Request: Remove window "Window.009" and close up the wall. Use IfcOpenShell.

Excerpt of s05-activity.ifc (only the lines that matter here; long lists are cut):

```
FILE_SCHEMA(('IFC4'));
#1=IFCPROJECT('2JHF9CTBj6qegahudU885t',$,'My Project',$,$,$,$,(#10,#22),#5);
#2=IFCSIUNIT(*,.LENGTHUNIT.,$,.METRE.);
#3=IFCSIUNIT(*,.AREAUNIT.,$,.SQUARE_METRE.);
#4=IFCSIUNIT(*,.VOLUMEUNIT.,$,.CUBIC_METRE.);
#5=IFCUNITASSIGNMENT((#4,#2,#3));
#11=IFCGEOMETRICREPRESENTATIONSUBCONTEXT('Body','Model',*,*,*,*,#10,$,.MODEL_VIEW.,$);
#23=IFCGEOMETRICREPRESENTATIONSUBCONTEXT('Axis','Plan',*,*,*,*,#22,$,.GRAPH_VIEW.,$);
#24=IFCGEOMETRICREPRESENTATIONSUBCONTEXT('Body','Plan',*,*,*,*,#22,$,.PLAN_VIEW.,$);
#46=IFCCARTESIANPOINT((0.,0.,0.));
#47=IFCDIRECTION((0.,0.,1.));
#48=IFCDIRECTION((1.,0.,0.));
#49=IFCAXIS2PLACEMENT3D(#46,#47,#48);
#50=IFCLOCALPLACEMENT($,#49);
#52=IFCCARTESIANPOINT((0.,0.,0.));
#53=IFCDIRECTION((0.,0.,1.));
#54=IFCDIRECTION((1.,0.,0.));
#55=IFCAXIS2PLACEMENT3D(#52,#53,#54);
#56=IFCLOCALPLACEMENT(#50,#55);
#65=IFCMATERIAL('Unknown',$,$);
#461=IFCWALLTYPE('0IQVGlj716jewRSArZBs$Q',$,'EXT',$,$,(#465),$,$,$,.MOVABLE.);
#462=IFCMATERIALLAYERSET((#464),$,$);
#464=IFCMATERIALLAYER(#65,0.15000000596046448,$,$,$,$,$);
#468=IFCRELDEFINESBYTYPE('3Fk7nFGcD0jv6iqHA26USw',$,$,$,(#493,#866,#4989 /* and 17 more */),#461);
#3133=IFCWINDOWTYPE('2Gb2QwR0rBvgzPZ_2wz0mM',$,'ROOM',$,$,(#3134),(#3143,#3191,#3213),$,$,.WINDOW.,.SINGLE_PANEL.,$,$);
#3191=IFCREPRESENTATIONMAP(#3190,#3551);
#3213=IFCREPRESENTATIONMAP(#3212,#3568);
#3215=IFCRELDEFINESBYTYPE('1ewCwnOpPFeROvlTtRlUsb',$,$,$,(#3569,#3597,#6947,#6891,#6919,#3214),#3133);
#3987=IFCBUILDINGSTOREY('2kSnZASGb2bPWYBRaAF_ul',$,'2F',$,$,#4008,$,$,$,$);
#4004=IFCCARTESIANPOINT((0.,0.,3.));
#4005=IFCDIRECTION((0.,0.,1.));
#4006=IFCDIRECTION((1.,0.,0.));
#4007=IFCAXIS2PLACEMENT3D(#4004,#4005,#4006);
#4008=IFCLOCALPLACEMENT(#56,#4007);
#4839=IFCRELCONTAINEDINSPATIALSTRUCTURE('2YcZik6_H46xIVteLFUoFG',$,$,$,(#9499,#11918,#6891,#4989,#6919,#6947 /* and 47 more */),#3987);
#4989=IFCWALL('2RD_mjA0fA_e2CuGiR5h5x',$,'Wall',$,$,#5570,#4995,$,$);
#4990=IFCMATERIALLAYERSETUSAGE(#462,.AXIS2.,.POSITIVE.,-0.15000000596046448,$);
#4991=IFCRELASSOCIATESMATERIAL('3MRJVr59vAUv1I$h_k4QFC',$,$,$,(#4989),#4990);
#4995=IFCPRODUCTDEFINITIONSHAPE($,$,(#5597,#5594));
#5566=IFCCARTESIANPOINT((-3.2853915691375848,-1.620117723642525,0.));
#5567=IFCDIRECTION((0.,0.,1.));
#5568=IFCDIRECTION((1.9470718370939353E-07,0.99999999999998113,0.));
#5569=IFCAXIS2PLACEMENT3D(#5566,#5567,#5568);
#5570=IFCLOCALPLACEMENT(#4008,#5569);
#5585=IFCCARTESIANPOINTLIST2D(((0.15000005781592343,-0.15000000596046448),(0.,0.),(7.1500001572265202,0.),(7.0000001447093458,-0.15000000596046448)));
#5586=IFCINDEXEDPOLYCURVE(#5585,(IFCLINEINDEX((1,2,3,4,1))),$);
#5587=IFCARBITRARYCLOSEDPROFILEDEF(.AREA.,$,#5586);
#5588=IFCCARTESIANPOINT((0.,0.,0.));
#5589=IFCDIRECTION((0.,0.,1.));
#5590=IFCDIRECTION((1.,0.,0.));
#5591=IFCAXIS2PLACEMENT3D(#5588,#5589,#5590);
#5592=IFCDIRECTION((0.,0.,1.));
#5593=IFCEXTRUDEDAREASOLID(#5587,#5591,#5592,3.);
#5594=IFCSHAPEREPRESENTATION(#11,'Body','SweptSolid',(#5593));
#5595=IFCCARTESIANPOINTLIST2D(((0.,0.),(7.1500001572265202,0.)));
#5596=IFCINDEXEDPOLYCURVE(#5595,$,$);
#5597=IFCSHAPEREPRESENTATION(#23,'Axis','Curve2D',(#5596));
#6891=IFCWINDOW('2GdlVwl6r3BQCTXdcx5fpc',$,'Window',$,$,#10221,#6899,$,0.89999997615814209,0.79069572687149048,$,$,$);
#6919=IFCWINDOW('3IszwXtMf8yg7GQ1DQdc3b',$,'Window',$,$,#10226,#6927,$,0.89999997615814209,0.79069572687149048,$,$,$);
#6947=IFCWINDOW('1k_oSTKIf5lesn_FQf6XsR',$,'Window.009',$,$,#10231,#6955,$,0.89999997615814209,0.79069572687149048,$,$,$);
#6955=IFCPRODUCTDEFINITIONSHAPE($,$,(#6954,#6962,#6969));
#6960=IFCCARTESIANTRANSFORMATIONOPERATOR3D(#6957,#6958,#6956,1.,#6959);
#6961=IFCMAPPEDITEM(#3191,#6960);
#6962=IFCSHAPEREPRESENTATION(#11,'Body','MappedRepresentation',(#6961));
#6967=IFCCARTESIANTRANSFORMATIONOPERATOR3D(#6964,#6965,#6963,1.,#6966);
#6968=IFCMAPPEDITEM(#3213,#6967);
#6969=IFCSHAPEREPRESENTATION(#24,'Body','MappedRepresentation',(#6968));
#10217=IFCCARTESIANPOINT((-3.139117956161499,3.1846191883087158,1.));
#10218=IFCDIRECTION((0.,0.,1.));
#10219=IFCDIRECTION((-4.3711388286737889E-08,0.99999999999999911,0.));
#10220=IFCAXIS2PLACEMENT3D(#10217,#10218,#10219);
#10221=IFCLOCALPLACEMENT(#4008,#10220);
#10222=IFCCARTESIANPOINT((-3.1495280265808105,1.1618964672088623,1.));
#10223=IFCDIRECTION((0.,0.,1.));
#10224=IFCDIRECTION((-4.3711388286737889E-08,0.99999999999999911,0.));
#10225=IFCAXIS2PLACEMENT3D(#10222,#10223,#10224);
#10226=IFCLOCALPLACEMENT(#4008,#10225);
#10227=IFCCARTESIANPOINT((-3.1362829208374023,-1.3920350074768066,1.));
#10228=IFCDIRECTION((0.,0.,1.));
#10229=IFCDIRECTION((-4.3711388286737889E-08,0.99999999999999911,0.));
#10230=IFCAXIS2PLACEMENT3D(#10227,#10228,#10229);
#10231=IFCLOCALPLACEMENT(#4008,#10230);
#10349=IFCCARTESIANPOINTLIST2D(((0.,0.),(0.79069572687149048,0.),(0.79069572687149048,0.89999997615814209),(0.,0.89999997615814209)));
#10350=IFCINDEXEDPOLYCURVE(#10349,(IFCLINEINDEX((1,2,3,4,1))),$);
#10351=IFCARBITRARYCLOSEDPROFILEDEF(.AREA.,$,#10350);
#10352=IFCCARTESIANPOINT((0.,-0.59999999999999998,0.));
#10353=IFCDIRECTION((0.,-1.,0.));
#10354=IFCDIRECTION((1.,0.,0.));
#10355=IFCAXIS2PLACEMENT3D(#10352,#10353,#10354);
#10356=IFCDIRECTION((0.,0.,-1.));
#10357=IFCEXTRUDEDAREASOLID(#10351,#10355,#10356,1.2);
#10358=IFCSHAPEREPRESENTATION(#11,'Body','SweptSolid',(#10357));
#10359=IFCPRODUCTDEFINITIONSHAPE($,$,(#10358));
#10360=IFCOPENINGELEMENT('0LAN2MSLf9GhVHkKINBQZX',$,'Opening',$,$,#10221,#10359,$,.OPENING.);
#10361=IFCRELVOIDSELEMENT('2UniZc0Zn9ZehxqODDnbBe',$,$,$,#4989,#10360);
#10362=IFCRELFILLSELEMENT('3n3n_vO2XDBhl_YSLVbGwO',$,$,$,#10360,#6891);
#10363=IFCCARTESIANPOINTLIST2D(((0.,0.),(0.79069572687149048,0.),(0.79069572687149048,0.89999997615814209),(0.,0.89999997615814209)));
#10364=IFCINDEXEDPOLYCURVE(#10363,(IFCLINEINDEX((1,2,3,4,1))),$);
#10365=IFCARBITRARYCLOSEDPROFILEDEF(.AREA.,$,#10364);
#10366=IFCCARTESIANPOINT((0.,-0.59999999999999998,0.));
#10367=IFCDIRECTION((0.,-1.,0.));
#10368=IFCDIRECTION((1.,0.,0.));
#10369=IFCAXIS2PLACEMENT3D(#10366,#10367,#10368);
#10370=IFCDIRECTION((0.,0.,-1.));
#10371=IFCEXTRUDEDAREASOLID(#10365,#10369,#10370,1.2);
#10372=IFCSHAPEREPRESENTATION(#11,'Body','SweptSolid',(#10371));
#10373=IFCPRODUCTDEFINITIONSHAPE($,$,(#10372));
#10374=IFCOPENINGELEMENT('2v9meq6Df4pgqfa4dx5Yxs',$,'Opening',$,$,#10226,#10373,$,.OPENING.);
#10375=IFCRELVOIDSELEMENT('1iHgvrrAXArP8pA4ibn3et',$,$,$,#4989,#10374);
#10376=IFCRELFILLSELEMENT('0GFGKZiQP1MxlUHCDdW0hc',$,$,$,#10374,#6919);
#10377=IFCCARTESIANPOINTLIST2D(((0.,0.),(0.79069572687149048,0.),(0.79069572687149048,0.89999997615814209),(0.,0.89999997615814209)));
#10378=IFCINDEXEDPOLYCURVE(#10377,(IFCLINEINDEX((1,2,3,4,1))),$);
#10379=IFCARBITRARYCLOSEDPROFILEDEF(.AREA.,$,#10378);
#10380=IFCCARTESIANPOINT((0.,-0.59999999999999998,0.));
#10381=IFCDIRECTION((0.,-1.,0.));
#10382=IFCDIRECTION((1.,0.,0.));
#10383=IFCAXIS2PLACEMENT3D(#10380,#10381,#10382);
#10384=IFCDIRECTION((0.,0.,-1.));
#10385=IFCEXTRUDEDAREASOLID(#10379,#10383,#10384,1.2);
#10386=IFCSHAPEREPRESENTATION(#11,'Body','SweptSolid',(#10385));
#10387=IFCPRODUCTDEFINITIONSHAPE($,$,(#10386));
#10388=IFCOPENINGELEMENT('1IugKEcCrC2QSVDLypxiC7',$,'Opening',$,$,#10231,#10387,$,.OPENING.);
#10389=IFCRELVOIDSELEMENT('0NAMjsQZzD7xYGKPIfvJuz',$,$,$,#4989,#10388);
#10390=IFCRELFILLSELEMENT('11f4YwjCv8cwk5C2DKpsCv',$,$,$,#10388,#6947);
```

```python
import ifcopenshell
import ifcopenshell.api.feature
import ifcopenshell.api.root
import ifcopenshell.geom
import ifcopenshell.util.shape

model = ifcopenshell.open("s05-activity.ifc")
settings = ifcopenshell.geom.settings()


def volume(element):
    """Net volume in cubic metres, openings subtracted."""
    shape = ifcopenshell.geom.create_shape(settings, element)
    return ifcopenshell.util.shape.get_volume(shape.geometry)


window = model.by_id(6947)
opening = window.FillsVoids[0].RelatingOpeningElement
wall = opening.VoidsElements[0].RelatingBuildingElement
before = volume(wall)

ifcopenshell.api.root.remove_product(model, product=window)
ifcopenshell.api.feature.remove_feature(model, feature=opening)

after = volume(wall)

print(f"wall volume {before:.3f} -> {after:.3f} m3")

model.write("s05-activity_v2.ifc")
```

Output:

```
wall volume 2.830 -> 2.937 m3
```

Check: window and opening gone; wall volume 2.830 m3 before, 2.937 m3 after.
